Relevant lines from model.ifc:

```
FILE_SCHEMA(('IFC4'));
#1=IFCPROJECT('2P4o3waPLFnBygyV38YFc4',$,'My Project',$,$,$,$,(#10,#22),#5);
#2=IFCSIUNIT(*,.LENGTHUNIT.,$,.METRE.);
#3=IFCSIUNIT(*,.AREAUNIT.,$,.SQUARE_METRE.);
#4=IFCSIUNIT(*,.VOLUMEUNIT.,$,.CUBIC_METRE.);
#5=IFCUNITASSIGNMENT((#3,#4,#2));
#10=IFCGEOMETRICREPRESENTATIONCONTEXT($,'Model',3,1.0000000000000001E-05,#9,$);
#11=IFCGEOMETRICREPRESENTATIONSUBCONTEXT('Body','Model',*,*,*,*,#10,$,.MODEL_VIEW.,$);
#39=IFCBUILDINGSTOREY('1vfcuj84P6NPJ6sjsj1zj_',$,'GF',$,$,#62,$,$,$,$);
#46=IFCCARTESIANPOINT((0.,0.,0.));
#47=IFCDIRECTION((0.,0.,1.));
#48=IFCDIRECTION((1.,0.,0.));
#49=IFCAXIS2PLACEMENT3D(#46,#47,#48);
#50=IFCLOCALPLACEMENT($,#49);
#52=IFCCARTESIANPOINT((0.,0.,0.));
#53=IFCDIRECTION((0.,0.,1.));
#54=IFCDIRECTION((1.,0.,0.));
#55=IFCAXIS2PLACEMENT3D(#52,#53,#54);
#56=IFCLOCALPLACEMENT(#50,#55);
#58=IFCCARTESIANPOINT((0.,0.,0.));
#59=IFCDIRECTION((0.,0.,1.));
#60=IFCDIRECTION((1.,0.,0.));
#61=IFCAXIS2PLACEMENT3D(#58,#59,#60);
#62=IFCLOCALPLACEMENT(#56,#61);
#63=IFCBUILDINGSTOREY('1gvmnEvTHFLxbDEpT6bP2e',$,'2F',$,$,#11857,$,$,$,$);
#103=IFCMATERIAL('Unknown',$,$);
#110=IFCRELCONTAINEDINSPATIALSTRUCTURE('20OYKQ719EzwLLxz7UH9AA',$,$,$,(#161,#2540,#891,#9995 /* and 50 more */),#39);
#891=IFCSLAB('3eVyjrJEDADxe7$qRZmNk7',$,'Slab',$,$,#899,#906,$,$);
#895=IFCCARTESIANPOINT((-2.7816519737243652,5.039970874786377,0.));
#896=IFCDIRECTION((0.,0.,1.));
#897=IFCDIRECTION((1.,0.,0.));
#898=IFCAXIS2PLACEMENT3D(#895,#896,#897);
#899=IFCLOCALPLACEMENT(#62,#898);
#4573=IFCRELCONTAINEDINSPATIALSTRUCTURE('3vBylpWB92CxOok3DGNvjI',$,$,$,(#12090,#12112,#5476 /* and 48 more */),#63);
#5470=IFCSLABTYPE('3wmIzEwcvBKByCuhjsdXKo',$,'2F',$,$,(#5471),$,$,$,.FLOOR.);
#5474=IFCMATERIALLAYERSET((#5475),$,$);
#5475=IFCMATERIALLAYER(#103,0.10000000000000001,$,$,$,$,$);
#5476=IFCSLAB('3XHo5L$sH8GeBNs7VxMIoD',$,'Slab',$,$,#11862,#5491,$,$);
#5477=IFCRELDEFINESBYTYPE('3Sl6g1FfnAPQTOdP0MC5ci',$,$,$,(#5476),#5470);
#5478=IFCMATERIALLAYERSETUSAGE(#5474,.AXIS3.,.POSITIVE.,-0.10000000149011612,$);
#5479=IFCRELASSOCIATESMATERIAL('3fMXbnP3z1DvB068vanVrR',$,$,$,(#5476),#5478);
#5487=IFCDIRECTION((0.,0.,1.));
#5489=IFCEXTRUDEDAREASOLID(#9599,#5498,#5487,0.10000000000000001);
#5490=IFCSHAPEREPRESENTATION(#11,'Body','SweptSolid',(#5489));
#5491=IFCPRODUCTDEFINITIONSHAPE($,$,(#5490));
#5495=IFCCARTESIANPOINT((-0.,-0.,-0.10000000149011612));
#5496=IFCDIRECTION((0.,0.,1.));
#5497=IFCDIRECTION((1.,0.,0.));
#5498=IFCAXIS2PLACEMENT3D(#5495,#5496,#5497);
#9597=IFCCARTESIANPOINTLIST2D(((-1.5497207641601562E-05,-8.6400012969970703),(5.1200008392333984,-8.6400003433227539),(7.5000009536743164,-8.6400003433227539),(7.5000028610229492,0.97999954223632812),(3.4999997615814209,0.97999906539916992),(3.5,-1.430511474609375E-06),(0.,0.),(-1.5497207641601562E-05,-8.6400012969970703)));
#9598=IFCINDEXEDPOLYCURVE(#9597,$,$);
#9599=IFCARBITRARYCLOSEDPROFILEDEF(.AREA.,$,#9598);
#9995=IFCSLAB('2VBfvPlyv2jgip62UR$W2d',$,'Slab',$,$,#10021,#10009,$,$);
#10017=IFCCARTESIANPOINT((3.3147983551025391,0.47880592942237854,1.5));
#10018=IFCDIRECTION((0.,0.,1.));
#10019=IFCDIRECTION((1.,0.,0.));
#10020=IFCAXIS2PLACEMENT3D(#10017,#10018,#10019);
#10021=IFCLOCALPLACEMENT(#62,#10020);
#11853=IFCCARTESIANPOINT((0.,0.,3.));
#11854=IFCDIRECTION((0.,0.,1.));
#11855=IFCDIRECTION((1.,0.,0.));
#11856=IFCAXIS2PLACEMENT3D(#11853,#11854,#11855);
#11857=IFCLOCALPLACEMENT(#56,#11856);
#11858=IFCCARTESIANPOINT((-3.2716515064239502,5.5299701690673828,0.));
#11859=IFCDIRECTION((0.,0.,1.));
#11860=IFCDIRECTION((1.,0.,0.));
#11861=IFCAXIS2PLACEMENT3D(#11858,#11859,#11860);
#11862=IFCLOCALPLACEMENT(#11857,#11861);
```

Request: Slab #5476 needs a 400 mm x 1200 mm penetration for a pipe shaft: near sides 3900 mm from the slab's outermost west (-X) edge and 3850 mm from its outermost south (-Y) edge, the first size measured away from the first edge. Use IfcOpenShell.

```python
import numpy as np
import ifcopenshell
import ifcopenshell.api.feature
import ifcopenshell.api.geometry
import ifcopenshell.api.root
import ifcopenshell.geom
import ifcopenshell.util.placement
import ifcopenshell.util.representation
import ifcopenshell.util.shape
import ifcopenshell.util.unit

model = ifcopenshell.open("model.ifc")
unit_scale = ifcopenshell.util.unit.calculate_unit_scale(model)
settings = ifcopenshell.geom.settings()


def volume(element):
    """Net volume in cubic metres, openings subtracted."""
    shape = ifcopenshell.geom.create_shape(settings, element)
    return ifcopenshell.util.shape.get_volume(shape.geometry)


slab = model.by_guid("3XHo5L$sH8GeBNs7VxMIoD")
before = volume(slab)

# Extent in the slab's own axes, in metres. The edges named are its -X and -Y sides.
slab_shape = ifcopenshell.geom.create_shape(settings, slab)
vertices = ifcopenshell.util.shape.get_vertices(slab_shape.geometry)
x_min, y_min, bottom = vertices.min(axis=0)
top = vertices[:, 2].max()

opening = ifcopenshell.api.root.create_entity(model, ifc_class="IfcOpeningElement", name="Pipe shaft opening", predefined_type="OPENING")
context = ifcopenshell.util.representation.get_context(model, "Model", "Body", "MODEL_VIEW")
width, depth = 0.4, 1.2
outline = [(0.0, 0.0), (width, 0.0), (width, depth), (0.0, depth), (0.0, 0.0)]
# Overshoot both faces by 50 mm so the cut is clean.
shape = ifcopenshell.api.geometry.add_slab_representation(
    model, context=context, depth=top - bottom + 0.1, polyline=outline
)
ifcopenshell.api.geometry.assign_representation(model, product=opening, representation=shape)

matrix = ifcopenshell.util.placement.get_local_placement(slab.ObjectPlacement)
matrix[:, 3] = matrix @ np.append(np.array([x_min + 3.9, y_min + 3.85, bottom - 0.05]) / unit_scale, 1.0)
ifcopenshell.api.geometry.edit_object_placement(model, product=opening, matrix=matrix, is_si=False)
ifcopenshell.api.feature.add_feature(model, feature=opening, element=slab)

after = volume(slab)

print(f"slab volume {before:.3f} -> {after:.3f} m3")

model.write("model_rev.ifc")
```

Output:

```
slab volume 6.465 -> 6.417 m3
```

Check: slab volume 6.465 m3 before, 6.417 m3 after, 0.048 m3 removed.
